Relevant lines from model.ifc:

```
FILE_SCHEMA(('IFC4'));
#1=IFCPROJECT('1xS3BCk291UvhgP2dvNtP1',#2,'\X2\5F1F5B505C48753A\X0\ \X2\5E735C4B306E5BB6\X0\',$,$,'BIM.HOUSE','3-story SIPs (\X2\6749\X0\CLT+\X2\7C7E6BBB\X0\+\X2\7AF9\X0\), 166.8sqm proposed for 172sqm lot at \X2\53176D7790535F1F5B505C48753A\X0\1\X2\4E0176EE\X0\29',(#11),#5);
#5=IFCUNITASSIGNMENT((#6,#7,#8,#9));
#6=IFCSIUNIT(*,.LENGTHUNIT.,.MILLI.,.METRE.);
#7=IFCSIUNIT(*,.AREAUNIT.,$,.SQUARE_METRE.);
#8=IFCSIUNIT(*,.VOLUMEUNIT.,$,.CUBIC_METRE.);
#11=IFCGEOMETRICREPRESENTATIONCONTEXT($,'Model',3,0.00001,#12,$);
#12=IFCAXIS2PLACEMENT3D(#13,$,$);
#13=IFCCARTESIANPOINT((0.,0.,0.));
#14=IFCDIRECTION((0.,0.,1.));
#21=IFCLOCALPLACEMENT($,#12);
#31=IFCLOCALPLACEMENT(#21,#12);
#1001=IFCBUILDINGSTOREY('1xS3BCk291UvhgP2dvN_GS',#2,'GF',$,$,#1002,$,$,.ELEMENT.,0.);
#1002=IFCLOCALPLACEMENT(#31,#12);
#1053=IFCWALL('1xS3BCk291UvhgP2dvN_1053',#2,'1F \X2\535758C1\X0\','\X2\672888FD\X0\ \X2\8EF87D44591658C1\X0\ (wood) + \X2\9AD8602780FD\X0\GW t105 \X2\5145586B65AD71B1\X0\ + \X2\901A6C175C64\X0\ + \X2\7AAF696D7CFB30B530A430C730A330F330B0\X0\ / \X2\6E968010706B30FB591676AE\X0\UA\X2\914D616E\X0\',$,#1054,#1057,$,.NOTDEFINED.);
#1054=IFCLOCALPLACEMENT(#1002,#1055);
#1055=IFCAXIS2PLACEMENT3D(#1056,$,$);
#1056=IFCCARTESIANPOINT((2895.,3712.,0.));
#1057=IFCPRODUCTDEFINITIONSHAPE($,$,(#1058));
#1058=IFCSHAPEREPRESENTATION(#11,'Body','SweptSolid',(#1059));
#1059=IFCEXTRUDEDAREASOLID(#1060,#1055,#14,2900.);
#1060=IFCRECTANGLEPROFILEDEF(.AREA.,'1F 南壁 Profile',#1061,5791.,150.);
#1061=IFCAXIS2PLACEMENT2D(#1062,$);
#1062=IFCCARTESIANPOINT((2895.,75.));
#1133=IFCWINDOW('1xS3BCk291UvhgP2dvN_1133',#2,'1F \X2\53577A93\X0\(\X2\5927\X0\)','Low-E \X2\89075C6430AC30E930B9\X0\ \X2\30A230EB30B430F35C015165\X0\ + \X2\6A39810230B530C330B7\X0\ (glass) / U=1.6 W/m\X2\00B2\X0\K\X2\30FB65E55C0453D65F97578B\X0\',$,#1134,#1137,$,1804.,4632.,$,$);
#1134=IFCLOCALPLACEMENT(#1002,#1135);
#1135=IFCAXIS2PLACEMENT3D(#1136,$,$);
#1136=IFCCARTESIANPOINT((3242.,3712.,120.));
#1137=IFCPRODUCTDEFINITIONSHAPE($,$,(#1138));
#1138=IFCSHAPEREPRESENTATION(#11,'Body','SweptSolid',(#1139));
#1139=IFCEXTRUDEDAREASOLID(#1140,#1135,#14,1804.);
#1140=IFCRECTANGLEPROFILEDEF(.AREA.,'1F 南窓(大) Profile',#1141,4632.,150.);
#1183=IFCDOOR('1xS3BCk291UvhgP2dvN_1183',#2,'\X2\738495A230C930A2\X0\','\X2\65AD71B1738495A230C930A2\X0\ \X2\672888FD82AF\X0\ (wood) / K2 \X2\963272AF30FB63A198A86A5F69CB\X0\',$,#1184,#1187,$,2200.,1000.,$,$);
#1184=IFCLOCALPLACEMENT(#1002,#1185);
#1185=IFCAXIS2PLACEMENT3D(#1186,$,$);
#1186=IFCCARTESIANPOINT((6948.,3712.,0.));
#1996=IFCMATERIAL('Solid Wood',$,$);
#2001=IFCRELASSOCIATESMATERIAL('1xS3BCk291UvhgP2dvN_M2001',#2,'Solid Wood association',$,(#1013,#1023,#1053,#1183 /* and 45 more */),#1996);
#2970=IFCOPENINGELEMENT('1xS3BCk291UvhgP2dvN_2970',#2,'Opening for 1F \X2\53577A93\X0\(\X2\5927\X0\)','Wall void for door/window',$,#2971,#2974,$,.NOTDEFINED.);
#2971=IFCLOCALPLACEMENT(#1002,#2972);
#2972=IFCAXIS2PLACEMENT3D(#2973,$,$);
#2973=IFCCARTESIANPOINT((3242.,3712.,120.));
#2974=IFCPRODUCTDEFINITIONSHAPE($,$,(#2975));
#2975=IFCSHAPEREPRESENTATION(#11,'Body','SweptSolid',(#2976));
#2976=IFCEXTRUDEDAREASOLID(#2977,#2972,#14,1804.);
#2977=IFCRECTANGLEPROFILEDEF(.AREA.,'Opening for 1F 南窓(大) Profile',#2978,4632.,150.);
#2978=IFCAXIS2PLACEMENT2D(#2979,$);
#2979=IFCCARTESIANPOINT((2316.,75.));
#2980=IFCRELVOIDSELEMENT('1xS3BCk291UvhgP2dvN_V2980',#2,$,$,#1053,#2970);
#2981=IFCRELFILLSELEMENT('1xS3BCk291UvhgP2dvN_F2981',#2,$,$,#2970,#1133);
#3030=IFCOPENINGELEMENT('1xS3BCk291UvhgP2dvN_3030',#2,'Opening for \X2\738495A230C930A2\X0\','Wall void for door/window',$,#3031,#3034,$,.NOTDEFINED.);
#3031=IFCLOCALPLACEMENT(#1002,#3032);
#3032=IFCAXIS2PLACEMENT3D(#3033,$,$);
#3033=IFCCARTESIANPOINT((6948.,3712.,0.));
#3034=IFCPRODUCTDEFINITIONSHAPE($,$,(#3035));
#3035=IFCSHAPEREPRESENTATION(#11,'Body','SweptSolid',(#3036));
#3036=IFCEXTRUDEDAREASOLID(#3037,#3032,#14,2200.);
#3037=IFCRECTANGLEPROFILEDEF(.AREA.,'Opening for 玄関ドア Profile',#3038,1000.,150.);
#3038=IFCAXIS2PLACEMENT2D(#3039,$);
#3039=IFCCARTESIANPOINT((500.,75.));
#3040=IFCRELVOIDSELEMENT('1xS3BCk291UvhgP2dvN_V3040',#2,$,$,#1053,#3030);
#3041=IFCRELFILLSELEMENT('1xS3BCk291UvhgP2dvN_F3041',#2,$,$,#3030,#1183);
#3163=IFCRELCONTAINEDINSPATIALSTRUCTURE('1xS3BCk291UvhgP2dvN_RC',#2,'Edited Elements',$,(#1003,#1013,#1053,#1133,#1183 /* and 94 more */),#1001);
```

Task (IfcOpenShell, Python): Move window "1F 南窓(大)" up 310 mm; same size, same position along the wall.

```python
import numpy as np
import ifcopenshell
import ifcopenshell.api.geometry
import ifcopenshell.util.placement
import ifcopenshell.util.unit

model = ifcopenshell.open("model.ifc")
unit_scale = ifcopenshell.util.unit.calculate_unit_scale(model)

window = model.by_guid("1xS3BCk291UvhgP2dvN_1133")
opening = window.FillsVoids[0].RelatingOpeningElement
dz = 310.0

shift = np.array([0.0, 0.0, dz])
# The window is not placed relative to its opening, so move both.
for product in (opening, window):
    matrix = ifcopenshell.util.placement.get_local_placement(product.ObjectPlacement)
    matrix[:3, 3] += shift
    ifcopenshell.api.geometry.edit_object_placement(model, product=product, matrix=matrix, is_si=False)

print(f"moved by {dz * unit_scale:+.3f} m")

model.write("model_edited.ifc")
```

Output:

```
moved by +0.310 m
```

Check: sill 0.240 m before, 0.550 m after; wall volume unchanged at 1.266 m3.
